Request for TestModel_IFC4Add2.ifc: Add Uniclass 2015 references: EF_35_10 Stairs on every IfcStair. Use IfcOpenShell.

First a look at what the model holds.

```python
import ifcopenshell

model = ifcopenshell.open("TestModel_IFC4Add2.ifc")
print(model.schema)
print("classifications:", [c.Name for c in model.by_type("IfcClassification")])
for ifc_class in ("IfcDoor", "IfcRoof", "IfcStair", "IfcWall", "IfcWindow"):
    print(ifc_class, len(model.by_type(ifc_class)))
```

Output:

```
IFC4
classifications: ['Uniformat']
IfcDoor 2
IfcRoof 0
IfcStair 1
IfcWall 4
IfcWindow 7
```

```python
import ifcopenshell
import ifcopenshell.api.classification

model = ifcopenshell.open("TestModel_IFC4Add2.ifc")

system = ifcopenshell.api.classification.add_classification(model, classification="Uniclass 2015")

codes = {
    "IfcStair": ("EF_35_10", "Stairs"),
}
for ifc_class, (code, name) in codes.items():
    products = model.by_type(ifc_class)
    ifcopenshell.api.classification.add_reference(
        model, products=products, classification=system, identification=code, name=name
    )
    print(code, len(products))

model.write("TestModel_IFC4Add2_v2.ifc")
```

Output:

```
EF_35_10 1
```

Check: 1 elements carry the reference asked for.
